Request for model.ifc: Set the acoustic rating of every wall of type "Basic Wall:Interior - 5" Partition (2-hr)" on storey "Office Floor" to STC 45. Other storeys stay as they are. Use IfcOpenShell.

First a look at what the model holds.

```python
import ifcopenshell
import ifcopenshell.util.element

model = ifcopenshell.open("model.ifc")
print(model.schema)
storey = next(s for s in model.by_type("IfcBuildingStorey") if s.Name == "Office Floor")
walls = [e for e in ifcopenshell.util.element.get_decomposition(storey) if e.is_a("IfcWall")]
seen = {}
for e in walls:
    element_type = ifcopenshell.util.element.get_type(e)
    key = (element_type.Name if element_type != e and element_type else None, ifcopenshell.util.element.get_pset(e, "Pset_WallCommon", "AcousticRating"))
    seen[key] = seen.get(key, 0) + 1
for (name, value), count in sorted(seen.items(), key=str):
    print(count, "x", name, "|", value)
```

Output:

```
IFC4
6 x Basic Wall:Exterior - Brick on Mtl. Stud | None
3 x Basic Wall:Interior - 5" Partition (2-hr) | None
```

```python
import ifcopenshell
import ifcopenshell.api.pset
import ifcopenshell.util.element

model = ifcopenshell.open("model.ifc")

storey = next(s for s in model.by_type("IfcBuildingStorey") if s.Name == "Office Floor")
walls = [e for e in ifcopenshell.util.element.get_decomposition(storey) if e.is_a("IfcWall")]

count = 0
for e in walls:
    element_type = ifcopenshell.util.element.get_type(e)
    if element_type in (None, e) or element_type.Name != 'Basic Wall:Interior - 5" Partition (2-hr)':
        continue
    # add_pset returns the element's existing set when there is one.
    pset = ifcopenshell.api.pset.add_pset(model, product=e, name="Pset_WallCommon")
    ifcopenshell.api.pset.edit_pset(model, pset=pset, properties={"AcousticRating": "STC 45"})
    count += 1

print(count, "walls updated")

model.write("model_edited.ifc")
```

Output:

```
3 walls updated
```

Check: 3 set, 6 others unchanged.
